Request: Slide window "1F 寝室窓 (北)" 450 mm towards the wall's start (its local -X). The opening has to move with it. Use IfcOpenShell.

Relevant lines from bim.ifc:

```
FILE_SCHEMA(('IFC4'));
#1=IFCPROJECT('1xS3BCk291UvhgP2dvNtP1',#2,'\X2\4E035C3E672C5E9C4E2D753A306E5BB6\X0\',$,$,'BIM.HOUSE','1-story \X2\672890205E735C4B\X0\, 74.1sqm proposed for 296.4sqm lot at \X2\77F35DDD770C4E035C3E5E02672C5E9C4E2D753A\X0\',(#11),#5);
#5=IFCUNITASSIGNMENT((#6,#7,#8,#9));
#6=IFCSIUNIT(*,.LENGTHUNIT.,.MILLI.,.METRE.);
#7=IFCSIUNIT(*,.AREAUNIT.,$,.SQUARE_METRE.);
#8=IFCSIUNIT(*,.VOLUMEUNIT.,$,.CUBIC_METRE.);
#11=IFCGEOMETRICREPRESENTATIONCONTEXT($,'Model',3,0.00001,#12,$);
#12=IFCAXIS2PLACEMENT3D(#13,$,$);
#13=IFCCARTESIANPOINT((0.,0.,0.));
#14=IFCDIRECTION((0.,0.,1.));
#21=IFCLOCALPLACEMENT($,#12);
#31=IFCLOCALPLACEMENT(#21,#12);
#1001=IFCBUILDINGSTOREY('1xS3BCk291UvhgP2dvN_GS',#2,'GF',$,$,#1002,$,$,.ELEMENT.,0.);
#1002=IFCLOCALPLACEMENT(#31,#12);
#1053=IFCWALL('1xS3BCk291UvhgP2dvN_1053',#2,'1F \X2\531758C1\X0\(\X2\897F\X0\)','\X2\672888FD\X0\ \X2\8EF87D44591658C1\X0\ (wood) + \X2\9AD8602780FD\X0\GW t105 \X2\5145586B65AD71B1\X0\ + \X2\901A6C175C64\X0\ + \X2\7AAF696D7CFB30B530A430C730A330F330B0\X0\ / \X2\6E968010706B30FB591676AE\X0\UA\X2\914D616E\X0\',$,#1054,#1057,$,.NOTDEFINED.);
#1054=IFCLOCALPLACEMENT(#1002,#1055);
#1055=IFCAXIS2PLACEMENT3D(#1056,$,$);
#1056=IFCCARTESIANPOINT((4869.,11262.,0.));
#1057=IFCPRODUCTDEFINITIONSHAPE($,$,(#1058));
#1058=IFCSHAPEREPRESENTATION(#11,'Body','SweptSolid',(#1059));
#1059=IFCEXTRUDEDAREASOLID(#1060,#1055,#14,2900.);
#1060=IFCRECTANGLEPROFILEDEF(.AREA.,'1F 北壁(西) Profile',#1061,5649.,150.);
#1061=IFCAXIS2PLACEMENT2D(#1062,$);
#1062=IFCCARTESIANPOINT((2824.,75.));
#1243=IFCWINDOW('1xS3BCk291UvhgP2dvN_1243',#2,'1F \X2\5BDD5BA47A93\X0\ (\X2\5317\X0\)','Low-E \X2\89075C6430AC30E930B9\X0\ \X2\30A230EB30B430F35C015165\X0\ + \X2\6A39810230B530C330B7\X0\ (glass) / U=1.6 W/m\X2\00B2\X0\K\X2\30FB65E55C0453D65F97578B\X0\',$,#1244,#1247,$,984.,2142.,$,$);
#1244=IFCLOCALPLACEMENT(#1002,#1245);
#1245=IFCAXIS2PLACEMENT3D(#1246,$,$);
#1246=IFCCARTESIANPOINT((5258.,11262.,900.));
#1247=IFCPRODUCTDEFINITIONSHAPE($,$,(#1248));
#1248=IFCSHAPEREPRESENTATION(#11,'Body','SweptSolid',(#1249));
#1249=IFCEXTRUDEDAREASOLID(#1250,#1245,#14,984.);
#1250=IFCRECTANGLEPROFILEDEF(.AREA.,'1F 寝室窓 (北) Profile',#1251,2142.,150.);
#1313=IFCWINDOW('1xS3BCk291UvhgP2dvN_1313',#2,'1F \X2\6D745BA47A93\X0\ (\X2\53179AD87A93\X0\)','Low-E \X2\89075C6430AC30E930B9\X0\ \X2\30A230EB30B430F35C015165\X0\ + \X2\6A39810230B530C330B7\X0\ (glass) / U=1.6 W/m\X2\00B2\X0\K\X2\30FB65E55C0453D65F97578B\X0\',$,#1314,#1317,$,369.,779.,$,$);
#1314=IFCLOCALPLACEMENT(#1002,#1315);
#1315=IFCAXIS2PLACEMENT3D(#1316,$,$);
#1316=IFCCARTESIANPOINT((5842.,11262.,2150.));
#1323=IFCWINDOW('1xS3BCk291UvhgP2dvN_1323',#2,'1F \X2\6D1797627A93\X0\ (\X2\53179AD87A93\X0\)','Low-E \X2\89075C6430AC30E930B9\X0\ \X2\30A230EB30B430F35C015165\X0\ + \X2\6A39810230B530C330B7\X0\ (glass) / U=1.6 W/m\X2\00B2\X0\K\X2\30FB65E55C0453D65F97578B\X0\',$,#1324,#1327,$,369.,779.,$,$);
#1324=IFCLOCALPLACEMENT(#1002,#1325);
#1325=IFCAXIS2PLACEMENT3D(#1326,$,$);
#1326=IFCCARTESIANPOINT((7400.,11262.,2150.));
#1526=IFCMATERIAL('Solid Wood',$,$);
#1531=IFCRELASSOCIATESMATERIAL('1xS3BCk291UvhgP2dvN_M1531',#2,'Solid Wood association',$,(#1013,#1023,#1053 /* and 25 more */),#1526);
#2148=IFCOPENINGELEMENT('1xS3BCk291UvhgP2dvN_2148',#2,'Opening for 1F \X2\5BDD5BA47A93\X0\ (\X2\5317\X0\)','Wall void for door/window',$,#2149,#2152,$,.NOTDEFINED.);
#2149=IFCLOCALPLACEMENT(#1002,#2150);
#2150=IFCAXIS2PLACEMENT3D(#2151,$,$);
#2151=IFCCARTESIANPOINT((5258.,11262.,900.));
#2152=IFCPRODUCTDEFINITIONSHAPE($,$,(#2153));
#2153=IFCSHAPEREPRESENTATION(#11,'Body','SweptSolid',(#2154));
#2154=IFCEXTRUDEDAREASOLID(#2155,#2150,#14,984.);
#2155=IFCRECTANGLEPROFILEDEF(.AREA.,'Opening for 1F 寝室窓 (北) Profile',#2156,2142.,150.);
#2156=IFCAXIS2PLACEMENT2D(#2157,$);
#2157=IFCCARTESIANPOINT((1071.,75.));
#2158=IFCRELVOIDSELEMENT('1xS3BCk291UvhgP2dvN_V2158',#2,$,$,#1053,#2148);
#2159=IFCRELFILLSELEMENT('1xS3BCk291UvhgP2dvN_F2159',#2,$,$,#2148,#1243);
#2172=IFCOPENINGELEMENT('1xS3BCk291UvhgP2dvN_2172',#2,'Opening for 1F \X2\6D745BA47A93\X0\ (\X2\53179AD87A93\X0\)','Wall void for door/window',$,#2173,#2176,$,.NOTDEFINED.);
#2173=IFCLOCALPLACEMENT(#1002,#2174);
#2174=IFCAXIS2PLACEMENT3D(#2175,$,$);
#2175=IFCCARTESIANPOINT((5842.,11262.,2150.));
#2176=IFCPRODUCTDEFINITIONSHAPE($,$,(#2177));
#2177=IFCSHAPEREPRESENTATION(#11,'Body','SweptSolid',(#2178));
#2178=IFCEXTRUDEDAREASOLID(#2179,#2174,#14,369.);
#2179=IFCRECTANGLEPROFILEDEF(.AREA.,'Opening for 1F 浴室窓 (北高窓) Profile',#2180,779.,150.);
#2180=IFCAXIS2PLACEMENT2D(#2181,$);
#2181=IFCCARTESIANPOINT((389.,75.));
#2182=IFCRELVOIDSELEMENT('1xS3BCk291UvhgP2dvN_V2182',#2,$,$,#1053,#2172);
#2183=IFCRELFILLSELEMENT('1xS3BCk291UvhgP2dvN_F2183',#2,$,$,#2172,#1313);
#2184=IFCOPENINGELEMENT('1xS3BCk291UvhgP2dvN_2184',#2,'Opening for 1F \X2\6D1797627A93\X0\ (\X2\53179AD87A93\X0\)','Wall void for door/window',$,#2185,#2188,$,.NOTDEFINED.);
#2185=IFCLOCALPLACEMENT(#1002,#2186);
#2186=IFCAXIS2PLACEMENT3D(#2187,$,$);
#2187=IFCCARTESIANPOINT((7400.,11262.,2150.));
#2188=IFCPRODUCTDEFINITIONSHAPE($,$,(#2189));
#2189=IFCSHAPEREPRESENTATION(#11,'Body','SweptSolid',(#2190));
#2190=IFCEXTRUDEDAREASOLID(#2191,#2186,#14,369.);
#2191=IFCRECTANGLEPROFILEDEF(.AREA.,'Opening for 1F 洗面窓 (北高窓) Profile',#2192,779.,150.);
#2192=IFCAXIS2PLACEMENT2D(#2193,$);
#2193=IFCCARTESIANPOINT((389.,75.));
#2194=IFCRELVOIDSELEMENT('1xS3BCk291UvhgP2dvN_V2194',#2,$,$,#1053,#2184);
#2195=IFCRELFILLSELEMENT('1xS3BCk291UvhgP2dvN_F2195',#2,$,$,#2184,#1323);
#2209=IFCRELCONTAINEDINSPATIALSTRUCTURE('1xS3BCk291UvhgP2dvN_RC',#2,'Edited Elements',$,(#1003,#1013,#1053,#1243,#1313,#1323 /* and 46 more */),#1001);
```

```python
import ifcopenshell
import ifcopenshell.api.geometry
import ifcopenshell.util.placement
import ifcopenshell.util.unit

model = ifcopenshell.open("bim.ifc")
unit_scale = ifcopenshell.util.unit.calculate_unit_scale(model)

window = model.by_id(1243)
opening = window.FillsVoids[0].RelatingOpeningElement
wall = opening.VoidsElements[0].RelatingBuildingElement

wall_matrix = ifcopenshell.util.placement.get_local_placement(wall.ObjectPlacement)
shift = wall_matrix[:3, 0] * -0.45 / unit_scale
before = ifcopenshell.util.placement.get_local_placement(window.ObjectPlacement)[:3, 3].copy()

# The window is not placed relative to its opening, so move both.
for product in (opening, window):
    matrix = ifcopenshell.util.placement.get_local_placement(product.ObjectPlacement)
    matrix[:3, 3] += shift
    ifcopenshell.api.geometry.edit_object_placement(model, product=product, matrix=matrix, is_si=False)

after = ifcopenshell.util.placement.get_local_placement(window.ObjectPlacement)[:3, 3]
print("window moved by", (after - before).round(3) + 0.0)

model.write("bim_updated.ifc")
```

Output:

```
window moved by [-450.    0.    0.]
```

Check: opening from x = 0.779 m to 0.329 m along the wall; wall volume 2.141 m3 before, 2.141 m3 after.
